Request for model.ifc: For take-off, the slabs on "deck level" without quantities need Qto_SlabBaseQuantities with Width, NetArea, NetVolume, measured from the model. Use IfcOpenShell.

First a look at what the model holds.

```python
import ifcopenshell
import ifcopenshell.util.element
import ifcopenshell.util.unit

model = ifcopenshell.open("model.ifc")
print(model.schema)
for unit_type in ("LENGTHUNIT", "AREAUNIT", "VOLUMEUNIT"):
    print(unit_type, ifcopenshell.util.unit.calculate_unit_scale(model, unit_type))
storey = next(s for s in model.by_type("IfcBuildingStorey") if s.Name == "deck level")
slabs = [e for e in ifcopenshell.util.element.get_decomposition(storey) if e.is_a("IfcSlab")]
for e in sorted(slabs, key=lambda e: e.id()):
    print(e.id(), e.is_a(), e.Name, list(ifcopenshell.util.element.get_psets(e, qtos_only=True)), sep=" | ")
```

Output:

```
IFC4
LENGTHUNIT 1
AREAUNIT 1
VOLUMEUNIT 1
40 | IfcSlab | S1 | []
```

```python
import ifcopenshell
import ifcopenshell.api.pset
import ifcopenshell.geom
import ifcopenshell.util.element
import ifcopenshell.util.shape
import ifcopenshell.util.unit

model = ifcopenshell.open("model.ifc")
unit_scale = ifcopenshell.util.unit.calculate_unit_scale(model)
area_scale = ifcopenshell.util.unit.calculate_unit_scale(model, "AREAUNIT")
volume_scale = ifcopenshell.util.unit.calculate_unit_scale(model, "VOLUMEUNIT")
settings = ifcopenshell.geom.settings()

storey = next(s for s in model.by_type("IfcBuildingStorey") if s.Name == "deck level")
slabs = [e for e in ifcopenshell.util.element.get_decomposition(storey) if e.is_a("IfcSlab")]

for e in sorted(slabs, key=lambda e: e.id()):
    if ifcopenshell.util.element.get_psets(e, qtos_only=True, should_inherit=False):
        continue
    # Geometry comes back in metres, in the element's own axes.
    shape = ifcopenshell.geom.create_shape(settings, e)
    values = {
        "Width": ifcopenshell.util.shape.get_z(shape.geometry) / unit_scale,
        "NetArea": ifcopenshell.util.shape.get_footprint_area(shape.geometry) / area_scale,
        "NetVolume": ifcopenshell.util.shape.get_volume(shape.geometry) / volume_scale,
    }
    qto = ifcopenshell.api.pset.add_qto(model, product=e, name="Qto_SlabBaseQuantities")
    ifcopenshell.api.pset.edit_qto(model, qto=qto, properties=values)
    print(e.id(), {k: round(v, 3) for k, v in values.items()})

model.write("model-out.ifc")
```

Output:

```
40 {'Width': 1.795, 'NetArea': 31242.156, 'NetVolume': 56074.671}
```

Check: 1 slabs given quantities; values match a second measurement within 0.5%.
